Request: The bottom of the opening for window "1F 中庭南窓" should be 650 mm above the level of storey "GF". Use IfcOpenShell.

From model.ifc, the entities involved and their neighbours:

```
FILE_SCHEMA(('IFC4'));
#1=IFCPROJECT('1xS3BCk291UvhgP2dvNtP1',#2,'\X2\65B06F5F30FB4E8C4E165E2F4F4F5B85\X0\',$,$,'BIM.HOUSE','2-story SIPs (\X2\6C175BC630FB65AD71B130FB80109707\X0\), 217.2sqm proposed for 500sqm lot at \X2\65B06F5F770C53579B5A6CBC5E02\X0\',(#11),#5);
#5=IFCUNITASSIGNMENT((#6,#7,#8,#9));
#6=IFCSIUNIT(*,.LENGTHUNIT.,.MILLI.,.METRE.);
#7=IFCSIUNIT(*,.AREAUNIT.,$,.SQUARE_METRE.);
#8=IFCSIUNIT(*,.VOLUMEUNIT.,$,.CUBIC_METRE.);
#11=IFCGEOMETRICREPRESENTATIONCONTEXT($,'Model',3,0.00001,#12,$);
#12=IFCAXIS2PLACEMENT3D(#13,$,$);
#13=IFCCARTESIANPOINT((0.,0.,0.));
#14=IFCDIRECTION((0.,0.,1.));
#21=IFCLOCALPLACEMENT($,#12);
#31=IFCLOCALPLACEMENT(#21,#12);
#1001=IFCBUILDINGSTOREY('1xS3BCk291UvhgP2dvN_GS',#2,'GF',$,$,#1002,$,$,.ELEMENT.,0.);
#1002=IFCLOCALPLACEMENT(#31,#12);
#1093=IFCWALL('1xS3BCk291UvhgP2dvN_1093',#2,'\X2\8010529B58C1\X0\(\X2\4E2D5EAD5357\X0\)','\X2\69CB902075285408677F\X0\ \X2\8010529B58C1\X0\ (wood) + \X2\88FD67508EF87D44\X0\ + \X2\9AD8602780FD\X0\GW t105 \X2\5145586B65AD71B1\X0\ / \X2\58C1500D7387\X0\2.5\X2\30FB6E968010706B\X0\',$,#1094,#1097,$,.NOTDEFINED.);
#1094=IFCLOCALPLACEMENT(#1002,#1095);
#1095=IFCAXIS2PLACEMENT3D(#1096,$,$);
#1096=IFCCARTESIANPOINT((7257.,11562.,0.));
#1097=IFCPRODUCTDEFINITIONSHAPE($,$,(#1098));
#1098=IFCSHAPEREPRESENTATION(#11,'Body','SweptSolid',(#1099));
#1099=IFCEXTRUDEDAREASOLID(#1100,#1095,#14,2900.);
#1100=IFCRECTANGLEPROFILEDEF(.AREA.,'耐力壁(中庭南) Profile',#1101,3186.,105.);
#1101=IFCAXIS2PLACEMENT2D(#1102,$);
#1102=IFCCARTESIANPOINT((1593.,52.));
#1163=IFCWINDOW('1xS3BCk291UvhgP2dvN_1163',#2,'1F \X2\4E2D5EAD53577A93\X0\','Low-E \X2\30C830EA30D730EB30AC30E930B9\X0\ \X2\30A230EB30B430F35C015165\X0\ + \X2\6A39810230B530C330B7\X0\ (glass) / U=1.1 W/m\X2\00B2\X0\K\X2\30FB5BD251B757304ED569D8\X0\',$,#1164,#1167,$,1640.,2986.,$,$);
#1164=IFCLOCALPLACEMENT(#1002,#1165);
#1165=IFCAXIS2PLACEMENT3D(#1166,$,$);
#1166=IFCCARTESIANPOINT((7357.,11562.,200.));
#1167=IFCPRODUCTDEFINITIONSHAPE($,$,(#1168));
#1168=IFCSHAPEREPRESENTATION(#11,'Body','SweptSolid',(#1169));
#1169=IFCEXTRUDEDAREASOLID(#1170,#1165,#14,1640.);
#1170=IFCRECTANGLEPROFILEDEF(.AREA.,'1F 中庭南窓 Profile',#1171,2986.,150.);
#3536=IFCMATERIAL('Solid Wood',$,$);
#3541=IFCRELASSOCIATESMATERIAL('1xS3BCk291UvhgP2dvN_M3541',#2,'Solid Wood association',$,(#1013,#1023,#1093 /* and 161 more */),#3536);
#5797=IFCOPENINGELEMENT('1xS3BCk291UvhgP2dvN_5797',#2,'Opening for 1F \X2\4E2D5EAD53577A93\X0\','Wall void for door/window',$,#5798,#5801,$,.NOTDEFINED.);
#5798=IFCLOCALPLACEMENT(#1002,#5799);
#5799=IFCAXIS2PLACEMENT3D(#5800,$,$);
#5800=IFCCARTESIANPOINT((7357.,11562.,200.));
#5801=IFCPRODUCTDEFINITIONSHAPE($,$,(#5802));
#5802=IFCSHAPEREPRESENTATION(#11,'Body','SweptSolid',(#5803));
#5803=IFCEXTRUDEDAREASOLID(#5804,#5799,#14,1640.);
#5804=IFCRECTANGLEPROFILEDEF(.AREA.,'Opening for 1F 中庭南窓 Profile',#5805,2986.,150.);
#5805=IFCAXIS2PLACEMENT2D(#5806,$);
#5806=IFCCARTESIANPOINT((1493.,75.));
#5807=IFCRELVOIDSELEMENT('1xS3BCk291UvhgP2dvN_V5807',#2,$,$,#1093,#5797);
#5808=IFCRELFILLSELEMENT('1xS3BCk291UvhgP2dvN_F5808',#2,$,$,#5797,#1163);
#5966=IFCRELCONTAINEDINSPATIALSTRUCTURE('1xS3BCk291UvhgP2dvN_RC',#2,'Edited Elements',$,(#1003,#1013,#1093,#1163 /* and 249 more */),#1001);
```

```python
import numpy as np
import ifcopenshell
import ifcopenshell.api.geometry
import ifcopenshell.geom
import ifcopenshell.util.element
import ifcopenshell.util.placement
import ifcopenshell.util.shape
import ifcopenshell.util.unit

model = ifcopenshell.open("model.ifc")
unit_scale = ifcopenshell.util.unit.calculate_unit_scale(model)

window = model.by_id(1163)
opening = window.FillsVoids[0].RelatingOpeningElement
storey = ifcopenshell.util.element.get_container(window, ifc_class="IfcBuildingStorey")
level = ifcopenshell.util.placement.get_local_placement(storey.ObjectPlacement)[2, 3]

# The opening's origin need not be at the sill, so measure its lowest point.
shape = ifcopenshell.geom.create_shape(ifcopenshell.geom.settings(), opening)
bottom = ifcopenshell.util.shape.get_shape_bottom_elevation(shape, shape.geometry) / unit_scale
dz = level + 650.0 - bottom

shift = np.array([0.0, 0.0, dz])
# The window is not placed relative to its opening, so move both.
for product in (opening, window):
    matrix = ifcopenshell.util.placement.get_local_placement(product.ObjectPlacement)
    matrix[:3, 3] += shift
    ifcopenshell.api.geometry.edit_object_placement(model, product=product, matrix=matrix, is_si=False)

print(f"moved by {dz * unit_scale:+.3f} m")

model.write("model_edited.ifc")
```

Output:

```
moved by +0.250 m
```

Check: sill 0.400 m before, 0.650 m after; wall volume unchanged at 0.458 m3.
